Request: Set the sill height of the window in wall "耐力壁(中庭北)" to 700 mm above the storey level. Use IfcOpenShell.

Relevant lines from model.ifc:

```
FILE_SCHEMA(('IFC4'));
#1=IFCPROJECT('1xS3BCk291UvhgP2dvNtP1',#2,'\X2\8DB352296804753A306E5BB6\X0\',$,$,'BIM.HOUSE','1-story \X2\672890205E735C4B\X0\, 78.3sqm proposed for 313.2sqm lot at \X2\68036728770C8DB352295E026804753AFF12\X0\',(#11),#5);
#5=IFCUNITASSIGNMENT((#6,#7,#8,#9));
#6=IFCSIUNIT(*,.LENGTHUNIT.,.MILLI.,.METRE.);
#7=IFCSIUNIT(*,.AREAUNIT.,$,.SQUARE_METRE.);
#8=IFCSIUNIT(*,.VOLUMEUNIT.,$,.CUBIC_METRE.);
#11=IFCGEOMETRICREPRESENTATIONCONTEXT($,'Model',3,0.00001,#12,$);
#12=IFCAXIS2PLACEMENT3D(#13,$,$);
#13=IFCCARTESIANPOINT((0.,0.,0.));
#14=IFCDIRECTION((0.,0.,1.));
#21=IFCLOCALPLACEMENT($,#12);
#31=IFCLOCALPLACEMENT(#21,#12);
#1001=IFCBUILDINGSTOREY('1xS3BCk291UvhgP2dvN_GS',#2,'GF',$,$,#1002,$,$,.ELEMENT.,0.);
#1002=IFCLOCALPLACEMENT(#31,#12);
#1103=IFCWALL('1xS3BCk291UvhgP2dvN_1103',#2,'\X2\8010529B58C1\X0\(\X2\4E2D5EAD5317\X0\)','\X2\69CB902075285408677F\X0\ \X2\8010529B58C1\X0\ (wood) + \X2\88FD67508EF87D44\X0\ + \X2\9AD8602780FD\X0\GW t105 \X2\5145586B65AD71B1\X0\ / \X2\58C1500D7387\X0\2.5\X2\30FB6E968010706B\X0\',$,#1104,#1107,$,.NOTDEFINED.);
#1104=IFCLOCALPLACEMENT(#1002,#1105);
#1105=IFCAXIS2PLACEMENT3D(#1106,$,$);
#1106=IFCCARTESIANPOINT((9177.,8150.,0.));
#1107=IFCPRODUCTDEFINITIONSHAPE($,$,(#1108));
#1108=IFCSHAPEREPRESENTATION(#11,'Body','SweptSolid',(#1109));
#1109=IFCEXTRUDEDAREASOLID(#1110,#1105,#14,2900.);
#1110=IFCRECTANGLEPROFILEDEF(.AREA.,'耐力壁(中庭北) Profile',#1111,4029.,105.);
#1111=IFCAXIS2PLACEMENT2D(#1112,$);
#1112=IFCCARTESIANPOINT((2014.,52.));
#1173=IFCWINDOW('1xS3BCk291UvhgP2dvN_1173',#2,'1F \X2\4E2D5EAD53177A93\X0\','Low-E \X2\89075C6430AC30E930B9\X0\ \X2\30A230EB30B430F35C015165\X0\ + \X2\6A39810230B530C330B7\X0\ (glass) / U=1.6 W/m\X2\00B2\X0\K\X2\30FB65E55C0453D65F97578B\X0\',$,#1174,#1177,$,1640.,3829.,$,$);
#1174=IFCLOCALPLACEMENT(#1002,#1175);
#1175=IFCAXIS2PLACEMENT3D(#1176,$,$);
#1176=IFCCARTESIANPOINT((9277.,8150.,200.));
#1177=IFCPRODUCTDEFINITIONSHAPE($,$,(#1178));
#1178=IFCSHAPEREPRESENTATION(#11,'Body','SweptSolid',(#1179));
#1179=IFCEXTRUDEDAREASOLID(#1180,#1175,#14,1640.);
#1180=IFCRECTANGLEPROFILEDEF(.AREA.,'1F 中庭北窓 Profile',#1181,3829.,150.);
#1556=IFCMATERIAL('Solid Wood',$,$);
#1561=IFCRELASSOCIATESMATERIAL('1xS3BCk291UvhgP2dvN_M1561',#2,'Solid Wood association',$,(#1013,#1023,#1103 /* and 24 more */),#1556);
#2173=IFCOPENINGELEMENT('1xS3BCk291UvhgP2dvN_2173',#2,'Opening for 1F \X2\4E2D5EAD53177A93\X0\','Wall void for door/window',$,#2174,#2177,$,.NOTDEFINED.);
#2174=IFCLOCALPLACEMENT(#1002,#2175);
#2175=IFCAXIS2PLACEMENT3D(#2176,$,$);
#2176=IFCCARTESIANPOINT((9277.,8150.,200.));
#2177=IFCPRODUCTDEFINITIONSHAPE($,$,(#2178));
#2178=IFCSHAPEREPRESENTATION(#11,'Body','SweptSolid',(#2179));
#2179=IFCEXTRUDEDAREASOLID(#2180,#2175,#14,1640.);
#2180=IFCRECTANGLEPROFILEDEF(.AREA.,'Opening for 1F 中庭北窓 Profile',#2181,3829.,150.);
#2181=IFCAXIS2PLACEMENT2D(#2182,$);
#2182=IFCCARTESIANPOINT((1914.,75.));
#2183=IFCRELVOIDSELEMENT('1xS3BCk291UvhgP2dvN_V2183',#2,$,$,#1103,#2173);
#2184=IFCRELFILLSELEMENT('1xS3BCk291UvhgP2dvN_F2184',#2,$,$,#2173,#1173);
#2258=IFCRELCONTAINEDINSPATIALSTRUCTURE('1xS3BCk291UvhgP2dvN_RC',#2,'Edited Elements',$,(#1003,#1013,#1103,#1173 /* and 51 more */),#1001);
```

```python
import numpy as np
import ifcopenshell
import ifcopenshell.api.geometry
import ifcopenshell.geom
import ifcopenshell.util.element
import ifcopenshell.util.placement
import ifcopenshell.util.shape
import ifcopenshell.util.unit

model = ifcopenshell.open("model.ifc")
unit_scale = ifcopenshell.util.unit.calculate_unit_scale(model)

window = model.by_guid("1xS3BCk291UvhgP2dvN_1173")
opening = window.FillsVoids[0].RelatingOpeningElement
storey = ifcopenshell.util.element.get_container(window, ifc_class="IfcBuildingStorey")
level = ifcopenshell.util.placement.get_local_placement(storey.ObjectPlacement)[2, 3]

# The opening's origin need not be at the sill, so measure its lowest point.
shape = ifcopenshell.geom.create_shape(ifcopenshell.geom.settings(), opening)
bottom = ifcopenshell.util.shape.get_shape_bottom_elevation(shape, shape.geometry) / unit_scale
dz = level + 700.0 - bottom

shift = np.array([0.0, 0.0, dz])
# The window is not placed relative to its opening, so move both.
for product in (opening, window):
    matrix = ifcopenshell.util.placement.get_local_placement(product.ObjectPlacement)
    matrix[:3, 3] += shift
    ifcopenshell.api.geometry.edit_object_placement(model, product=product, matrix=matrix, is_si=False)

print(f"moved by {dz * unit_scale:+.3f} m")

model.write("model-out.ifc")
```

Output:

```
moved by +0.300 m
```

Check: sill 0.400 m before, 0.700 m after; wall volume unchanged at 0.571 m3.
